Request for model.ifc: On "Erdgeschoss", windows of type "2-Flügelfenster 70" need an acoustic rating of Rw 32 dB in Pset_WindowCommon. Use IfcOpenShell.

First a look at what the model holds.

```python
import ifcopenshell
import ifcopenshell.util.element

model = ifcopenshell.open("model.ifc")
print(model.schema)
storey = next(s for s in model.by_type("IfcBuildingStorey") if s.Name == "Erdgeschoss")
windows = [e for e in ifcopenshell.util.element.get_decomposition(storey) if e.is_a("IfcWindow")]
seen = {}
for e in windows:
    element_type = ifcopenshell.util.element.get_type(e)
    key = (element_type.Name if element_type != e and element_type else None, ifcopenshell.util.element.get_pset(e, "Pset_WindowCommon", "AcousticRating"))
    seen[key] = seen.get(key, 0) + 1
for (name, value), count in sorted(seen.items(), key=str):
    print(count, "x", name, "|", value)
```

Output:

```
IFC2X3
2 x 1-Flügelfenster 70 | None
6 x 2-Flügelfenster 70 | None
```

```python
import ifcopenshell
import ifcopenshell.api.pset
import ifcopenshell.util.element

model = ifcopenshell.open("model.ifc")

storey = next(s for s in model.by_type("IfcBuildingStorey") if s.Name == "Erdgeschoss")
windows = [e for e in ifcopenshell.util.element.get_decomposition(storey) if e.is_a("IfcWindow")]

count = 0
for e in windows:
    element_type = ifcopenshell.util.element.get_type(e)
    if element_type in (None, e) or element_type.Name != "2-Flügelfenster 70":
        continue
    # add_pset returns the element's existing set when there is one.
    pset = ifcopenshell.api.pset.add_pset(model, product=e, name="Pset_WindowCommon")
    ifcopenshell.api.pset.edit_pset(model, pset=pset, properties={"AcousticRating": "Rw 32 dB"})
    count += 1

print(count, "windows updated")

model.write("model_v2.ifc")
```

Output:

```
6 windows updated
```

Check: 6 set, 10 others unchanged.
